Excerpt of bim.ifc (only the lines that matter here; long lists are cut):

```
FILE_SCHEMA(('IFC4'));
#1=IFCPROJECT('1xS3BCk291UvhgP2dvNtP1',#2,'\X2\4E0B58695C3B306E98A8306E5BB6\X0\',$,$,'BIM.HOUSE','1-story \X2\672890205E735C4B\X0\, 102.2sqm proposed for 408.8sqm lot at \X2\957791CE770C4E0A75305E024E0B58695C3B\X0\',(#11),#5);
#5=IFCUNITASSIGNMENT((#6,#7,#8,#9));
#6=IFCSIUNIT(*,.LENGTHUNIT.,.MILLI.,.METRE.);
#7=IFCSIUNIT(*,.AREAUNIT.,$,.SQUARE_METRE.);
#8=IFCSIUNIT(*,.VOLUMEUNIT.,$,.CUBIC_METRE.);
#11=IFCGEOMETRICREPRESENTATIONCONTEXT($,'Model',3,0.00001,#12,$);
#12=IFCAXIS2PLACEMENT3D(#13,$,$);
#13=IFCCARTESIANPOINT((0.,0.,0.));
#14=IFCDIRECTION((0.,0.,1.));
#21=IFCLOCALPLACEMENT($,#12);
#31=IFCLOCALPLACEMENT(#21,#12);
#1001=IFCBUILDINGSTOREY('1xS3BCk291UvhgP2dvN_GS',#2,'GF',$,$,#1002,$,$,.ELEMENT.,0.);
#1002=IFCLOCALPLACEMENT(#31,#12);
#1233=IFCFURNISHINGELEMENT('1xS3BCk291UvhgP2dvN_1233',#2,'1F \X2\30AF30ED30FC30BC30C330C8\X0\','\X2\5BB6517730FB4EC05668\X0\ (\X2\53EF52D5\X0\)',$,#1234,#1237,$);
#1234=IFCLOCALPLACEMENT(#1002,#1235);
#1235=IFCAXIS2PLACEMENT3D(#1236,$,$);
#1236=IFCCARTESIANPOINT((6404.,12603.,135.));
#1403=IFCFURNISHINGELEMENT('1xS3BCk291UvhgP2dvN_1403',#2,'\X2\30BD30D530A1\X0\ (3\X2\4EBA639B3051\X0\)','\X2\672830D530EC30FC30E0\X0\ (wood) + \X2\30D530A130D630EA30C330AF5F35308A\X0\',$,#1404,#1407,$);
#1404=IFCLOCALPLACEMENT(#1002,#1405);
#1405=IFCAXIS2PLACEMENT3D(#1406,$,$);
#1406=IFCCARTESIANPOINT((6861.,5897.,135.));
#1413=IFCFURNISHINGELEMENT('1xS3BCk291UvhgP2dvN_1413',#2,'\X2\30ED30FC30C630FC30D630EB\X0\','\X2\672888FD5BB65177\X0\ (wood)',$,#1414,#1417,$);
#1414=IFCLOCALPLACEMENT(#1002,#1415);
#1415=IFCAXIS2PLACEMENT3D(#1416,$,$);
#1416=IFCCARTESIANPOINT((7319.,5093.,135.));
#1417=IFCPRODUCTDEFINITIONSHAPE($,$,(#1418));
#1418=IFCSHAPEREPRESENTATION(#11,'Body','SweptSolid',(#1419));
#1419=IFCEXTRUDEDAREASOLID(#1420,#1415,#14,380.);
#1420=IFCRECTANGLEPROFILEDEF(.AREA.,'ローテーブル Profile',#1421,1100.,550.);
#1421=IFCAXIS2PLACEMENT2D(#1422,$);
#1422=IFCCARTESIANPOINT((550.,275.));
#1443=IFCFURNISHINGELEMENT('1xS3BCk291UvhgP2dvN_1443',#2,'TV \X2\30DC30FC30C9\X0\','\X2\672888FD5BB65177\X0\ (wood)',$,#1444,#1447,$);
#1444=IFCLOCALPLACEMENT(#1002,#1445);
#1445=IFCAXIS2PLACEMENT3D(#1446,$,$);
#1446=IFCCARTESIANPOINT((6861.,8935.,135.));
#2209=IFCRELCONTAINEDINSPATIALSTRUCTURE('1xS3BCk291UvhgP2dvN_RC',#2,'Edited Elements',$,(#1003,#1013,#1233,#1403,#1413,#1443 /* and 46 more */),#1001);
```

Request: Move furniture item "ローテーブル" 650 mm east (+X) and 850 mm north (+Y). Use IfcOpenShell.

```python
import ifcopenshell
import ifcopenshell.api.geometry
import ifcopenshell.util.placement

model = ifcopenshell.open("bim.ifc")

item = model.by_id(1413)
matrix = ifcopenshell.util.placement.get_local_placement(item.ObjectPlacement)
matrix[0, 3] += 650.0
matrix[1, 3] += 850.0
ifcopenshell.api.geometry.edit_object_placement(model, product=item, matrix=matrix, is_si=False)

print(ifcopenshell.util.placement.get_local_placement(item.ObjectPlacement).round(3) + 0.0)

model.write("bim_v2.ifc")
```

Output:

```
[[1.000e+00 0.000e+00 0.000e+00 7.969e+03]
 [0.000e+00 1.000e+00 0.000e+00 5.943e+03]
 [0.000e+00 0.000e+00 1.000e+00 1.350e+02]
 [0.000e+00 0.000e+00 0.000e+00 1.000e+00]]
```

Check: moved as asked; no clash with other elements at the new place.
